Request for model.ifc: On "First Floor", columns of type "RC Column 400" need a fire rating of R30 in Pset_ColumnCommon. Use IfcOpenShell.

First a look at what the model holds.

```python
import ifcopenshell
import ifcopenshell.util.element

model = ifcopenshell.open("model.ifc")
print(model.schema)
storey = next(s for s in model.by_type("IfcBuildingStorey") if s.Name == "First Floor")
columns = [e for e in ifcopenshell.util.element.get_decomposition(storey) if e.is_a("IfcColumn")]
seen = {}
for e in columns:
    element_type = ifcopenshell.util.element.get_type(e)
    key = (element_type.Name if element_type != e and element_type else None, ifcopenshell.util.element.get_pset(e, "Pset_ColumnCommon", "FireRating"))
    seen[key] = seen.get(key, 0) + 1
for (name, value), count in sorted(seen.items(), key=str):
    print(count, "x", name, "|", value)
```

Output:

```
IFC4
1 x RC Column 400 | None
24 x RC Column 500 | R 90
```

```python
import ifcopenshell
import ifcopenshell.api.pset
import ifcopenshell.util.element

model = ifcopenshell.open("model.ifc")

storey = next(s for s in model.by_type("IfcBuildingStorey") if s.Name == "First Floor")
columns = [e for e in ifcopenshell.util.element.get_decomposition(storey) if e.is_a("IfcColumn")]

count = 0
for e in columns:
    element_type = ifcopenshell.util.element.get_type(e)
    if element_type in (None, e) or element_type.Name != "RC Column 400":
        continue
    # add_pset returns the element's existing set when there is one.
    pset = ifcopenshell.api.pset.add_pset(model, product=e, name="Pset_ColumnCommon")
    ifcopenshell.api.pset.edit_pset(model, pset=pset, properties={"FireRating": "R30"})
    count += 1

print(count, "columns updated")

model.write("model_rev.ifc")
```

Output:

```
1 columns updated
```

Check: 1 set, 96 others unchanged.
